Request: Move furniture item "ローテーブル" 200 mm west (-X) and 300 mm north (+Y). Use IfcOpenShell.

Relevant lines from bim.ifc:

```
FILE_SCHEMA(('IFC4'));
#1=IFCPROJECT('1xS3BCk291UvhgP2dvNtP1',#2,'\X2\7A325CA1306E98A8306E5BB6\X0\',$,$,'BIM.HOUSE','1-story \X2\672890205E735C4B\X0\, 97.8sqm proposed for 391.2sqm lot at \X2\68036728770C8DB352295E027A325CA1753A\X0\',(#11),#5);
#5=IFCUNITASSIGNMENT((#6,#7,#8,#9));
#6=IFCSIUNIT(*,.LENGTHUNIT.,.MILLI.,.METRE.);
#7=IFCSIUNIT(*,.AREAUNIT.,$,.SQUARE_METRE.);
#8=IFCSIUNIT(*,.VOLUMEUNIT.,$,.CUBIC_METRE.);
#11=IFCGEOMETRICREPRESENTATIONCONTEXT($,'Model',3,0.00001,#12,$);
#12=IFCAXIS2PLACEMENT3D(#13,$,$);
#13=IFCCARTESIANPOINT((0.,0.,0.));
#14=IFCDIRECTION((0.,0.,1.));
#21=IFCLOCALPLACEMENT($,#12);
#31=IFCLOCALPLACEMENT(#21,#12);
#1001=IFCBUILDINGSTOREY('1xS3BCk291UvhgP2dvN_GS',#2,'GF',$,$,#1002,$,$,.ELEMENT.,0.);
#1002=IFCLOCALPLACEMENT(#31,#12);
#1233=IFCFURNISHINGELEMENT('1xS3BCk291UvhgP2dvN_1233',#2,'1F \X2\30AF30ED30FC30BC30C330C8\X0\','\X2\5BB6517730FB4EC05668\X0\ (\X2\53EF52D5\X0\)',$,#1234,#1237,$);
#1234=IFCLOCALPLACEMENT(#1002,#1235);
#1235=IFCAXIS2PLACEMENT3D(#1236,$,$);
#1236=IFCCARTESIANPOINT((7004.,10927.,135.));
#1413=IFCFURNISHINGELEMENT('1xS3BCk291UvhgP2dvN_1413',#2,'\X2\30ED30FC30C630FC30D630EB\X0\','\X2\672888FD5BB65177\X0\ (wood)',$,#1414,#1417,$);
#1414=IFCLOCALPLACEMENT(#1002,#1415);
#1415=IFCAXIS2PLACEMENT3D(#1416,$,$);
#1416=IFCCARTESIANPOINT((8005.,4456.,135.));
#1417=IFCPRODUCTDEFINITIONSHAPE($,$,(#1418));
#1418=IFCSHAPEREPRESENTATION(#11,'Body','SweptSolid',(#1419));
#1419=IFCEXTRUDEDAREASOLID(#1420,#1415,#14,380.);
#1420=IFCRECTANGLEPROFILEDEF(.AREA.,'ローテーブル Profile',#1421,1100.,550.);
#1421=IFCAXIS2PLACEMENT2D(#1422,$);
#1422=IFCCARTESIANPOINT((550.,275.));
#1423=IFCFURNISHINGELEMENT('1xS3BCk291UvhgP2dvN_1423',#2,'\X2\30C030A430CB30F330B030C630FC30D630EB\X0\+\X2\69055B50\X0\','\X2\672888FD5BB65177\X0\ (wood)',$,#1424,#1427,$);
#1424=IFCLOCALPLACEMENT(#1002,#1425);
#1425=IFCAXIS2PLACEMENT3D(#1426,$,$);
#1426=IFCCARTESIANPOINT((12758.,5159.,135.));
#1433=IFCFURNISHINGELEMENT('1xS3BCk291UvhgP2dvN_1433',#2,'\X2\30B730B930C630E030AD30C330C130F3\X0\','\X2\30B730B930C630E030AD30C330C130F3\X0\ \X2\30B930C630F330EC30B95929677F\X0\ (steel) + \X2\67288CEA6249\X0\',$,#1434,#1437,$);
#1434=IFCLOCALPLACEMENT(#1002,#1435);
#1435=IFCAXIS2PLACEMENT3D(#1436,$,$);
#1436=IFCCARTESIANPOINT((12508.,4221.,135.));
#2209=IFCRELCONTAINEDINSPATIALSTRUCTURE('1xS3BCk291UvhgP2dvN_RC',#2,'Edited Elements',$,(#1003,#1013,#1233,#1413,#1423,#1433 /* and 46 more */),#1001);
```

```python
import ifcopenshell
import ifcopenshell.api.geometry
import ifcopenshell.util.placement
import ifcopenshell.util.unit

model = ifcopenshell.open("bim.ifc")
unit_scale = ifcopenshell.util.unit.calculate_unit_scale(model)

item = model.by_id(1413)
matrix = ifcopenshell.util.placement.get_local_placement(item.ObjectPlacement)
matrix[0, 3] -= 0.2 / unit_scale
matrix[1, 3] += 0.3 / unit_scale
ifcopenshell.api.geometry.edit_object_placement(model, product=item, matrix=matrix, is_si=False)

print(ifcopenshell.util.placement.get_local_placement(item.ObjectPlacement).round(3) + 0.0)

model.write("bim_updated.ifc")
```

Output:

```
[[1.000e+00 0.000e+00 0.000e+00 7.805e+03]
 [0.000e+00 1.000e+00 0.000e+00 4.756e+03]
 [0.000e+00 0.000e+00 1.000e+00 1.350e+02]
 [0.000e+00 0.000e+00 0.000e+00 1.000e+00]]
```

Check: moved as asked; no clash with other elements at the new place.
